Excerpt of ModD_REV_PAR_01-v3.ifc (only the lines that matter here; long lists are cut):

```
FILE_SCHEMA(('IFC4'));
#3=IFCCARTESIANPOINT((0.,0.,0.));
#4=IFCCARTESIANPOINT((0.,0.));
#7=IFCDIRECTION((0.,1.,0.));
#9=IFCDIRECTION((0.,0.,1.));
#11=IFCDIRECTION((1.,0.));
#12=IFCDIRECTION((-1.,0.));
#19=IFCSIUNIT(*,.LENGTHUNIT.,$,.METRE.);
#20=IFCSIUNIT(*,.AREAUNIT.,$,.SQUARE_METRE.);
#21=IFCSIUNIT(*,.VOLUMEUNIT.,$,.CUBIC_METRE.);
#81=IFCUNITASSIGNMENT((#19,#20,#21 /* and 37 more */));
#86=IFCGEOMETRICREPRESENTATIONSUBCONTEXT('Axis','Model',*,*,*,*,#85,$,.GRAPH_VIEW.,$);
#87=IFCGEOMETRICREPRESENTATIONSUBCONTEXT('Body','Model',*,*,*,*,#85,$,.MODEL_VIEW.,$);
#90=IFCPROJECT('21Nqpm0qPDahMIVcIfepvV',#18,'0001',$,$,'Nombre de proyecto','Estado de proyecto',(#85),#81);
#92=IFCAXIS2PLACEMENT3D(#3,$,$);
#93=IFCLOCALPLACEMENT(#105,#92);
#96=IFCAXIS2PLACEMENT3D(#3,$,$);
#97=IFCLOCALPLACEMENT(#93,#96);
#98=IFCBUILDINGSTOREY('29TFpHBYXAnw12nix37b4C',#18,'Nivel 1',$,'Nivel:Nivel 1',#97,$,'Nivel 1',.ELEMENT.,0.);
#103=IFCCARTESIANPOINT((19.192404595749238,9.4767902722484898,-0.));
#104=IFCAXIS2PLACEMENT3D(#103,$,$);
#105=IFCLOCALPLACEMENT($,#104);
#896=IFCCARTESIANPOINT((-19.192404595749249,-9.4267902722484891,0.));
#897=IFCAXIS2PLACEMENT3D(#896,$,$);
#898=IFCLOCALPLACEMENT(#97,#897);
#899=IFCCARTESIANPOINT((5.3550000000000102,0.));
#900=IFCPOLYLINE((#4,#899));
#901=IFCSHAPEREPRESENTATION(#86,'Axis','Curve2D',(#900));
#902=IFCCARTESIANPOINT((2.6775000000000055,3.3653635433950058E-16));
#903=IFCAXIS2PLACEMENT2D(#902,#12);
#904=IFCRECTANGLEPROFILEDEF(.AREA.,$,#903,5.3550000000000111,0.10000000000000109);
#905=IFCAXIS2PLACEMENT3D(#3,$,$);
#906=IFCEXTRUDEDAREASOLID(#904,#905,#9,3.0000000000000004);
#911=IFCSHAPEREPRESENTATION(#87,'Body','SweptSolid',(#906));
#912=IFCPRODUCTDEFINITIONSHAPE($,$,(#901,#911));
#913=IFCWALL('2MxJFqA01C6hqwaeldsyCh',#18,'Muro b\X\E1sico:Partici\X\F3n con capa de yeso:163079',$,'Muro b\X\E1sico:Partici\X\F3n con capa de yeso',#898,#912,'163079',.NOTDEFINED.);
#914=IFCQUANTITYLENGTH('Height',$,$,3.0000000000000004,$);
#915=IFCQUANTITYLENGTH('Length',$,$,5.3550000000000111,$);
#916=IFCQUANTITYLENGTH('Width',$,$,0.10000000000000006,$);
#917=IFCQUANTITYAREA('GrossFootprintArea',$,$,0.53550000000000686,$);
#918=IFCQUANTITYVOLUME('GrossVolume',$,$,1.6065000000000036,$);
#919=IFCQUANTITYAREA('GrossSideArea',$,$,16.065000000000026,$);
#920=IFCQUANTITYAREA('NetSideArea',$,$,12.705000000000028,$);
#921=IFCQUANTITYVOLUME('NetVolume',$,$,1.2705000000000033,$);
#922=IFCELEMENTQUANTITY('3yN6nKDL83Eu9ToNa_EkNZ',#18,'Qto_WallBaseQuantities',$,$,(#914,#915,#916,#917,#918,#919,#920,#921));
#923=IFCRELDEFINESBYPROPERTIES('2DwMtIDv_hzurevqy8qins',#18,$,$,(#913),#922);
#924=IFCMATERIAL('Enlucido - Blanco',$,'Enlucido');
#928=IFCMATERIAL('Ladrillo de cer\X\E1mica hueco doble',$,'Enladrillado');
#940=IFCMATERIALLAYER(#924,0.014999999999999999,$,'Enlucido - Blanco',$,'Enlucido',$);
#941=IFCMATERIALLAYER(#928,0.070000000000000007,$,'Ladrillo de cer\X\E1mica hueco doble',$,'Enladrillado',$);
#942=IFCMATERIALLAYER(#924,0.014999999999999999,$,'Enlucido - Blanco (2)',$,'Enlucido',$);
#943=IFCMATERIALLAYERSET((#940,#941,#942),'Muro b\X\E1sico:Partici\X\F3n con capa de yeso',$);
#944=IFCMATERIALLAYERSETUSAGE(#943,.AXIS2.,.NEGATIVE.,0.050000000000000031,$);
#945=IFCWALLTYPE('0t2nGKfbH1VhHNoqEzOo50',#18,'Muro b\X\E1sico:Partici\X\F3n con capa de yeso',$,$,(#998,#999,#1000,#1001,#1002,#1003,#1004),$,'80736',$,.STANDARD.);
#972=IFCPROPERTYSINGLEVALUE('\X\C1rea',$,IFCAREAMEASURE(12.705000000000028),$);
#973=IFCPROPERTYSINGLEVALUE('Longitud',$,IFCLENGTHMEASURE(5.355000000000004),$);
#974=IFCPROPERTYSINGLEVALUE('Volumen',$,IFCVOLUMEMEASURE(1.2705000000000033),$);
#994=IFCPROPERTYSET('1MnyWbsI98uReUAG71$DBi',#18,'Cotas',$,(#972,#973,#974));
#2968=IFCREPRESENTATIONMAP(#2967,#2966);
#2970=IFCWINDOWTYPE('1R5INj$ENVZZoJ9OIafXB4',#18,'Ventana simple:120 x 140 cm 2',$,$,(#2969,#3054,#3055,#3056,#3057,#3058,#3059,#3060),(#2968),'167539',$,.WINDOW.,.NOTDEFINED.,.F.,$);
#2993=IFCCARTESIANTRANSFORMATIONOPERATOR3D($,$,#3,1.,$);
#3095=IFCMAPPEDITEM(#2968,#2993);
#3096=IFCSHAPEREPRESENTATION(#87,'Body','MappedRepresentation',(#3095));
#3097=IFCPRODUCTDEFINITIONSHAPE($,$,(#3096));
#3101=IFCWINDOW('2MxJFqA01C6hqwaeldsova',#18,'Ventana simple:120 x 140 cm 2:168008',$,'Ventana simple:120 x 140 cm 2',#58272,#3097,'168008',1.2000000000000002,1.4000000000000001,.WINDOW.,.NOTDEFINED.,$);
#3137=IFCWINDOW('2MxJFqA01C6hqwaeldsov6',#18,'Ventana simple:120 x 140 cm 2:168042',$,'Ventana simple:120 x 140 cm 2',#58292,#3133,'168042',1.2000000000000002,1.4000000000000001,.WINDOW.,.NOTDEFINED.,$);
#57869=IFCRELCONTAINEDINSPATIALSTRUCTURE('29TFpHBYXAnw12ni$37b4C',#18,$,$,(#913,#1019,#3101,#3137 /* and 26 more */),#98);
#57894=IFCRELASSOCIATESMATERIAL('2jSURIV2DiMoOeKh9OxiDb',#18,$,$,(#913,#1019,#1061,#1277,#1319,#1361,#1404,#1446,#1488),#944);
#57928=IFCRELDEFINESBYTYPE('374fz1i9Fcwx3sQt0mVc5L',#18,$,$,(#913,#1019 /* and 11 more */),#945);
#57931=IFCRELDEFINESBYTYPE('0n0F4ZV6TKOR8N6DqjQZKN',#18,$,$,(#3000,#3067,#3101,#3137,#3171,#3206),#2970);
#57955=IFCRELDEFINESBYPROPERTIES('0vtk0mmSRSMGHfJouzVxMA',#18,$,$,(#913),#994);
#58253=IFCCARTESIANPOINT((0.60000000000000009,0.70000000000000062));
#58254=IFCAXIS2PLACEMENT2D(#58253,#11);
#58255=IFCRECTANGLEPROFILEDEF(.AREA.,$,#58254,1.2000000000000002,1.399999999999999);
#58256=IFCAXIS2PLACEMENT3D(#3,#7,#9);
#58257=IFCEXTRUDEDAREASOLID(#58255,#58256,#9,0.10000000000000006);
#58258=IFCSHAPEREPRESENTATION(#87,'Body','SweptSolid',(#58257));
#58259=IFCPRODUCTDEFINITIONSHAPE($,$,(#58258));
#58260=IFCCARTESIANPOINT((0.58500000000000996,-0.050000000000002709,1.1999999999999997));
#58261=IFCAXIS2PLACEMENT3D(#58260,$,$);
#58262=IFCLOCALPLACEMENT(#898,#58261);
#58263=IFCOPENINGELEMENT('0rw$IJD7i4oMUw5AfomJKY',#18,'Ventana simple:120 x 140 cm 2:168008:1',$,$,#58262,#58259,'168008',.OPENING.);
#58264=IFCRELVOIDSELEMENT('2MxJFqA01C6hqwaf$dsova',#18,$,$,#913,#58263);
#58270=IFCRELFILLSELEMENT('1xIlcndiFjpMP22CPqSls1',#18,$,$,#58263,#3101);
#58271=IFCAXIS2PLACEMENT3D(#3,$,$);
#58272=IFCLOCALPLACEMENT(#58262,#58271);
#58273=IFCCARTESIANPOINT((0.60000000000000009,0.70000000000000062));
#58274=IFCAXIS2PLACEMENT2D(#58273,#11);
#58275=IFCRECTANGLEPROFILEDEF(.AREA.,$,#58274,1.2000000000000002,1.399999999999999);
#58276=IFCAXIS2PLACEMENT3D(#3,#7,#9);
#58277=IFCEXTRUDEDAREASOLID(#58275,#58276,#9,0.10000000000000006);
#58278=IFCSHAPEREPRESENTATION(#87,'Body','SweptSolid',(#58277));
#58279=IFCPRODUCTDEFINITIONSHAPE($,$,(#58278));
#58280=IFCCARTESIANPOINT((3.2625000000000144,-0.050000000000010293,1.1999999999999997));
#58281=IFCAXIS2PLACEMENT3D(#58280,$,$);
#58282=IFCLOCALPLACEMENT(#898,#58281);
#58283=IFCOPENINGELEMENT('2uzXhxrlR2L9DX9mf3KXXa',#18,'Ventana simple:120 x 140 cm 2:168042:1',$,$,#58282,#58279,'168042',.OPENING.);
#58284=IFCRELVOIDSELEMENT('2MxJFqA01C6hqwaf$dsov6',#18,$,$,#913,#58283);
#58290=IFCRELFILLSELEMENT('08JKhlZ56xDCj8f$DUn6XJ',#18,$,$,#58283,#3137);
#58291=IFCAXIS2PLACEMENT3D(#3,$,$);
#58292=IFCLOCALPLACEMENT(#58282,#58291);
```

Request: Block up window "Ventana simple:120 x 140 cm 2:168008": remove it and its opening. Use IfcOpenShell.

```python
import ifcopenshell
import ifcopenshell.api.feature
import ifcopenshell.api.pset
import ifcopenshell.api.root
import ifcopenshell.geom
import ifcopenshell.util.element
import ifcopenshell.util.shape
import ifcopenshell.util.unit

model = ifcopenshell.open("ModD_REV_PAR_01-v3.ifc")
area_scale = ifcopenshell.util.unit.calculate_unit_scale(model, "AREAUNIT")
volume_scale = ifcopenshell.util.unit.calculate_unit_scale(model, "VOLUMEUNIT")
settings = ifcopenshell.geom.settings()


def volume(element):
    """Net volume in cubic metres, openings subtracted."""
    shape = ifcopenshell.geom.create_shape(settings, element)
    return ifcopenshell.util.shape.get_volume(shape.geometry)


window = model.by_id(3101)
opening = window.FillsVoids[0].RelatingOpeningElement
wall = opening.VoidsElements[0].RelatingBuildingElement
before = volume(wall)

ifcopenshell.api.root.remove_product(model, product=window)
ifcopenshell.api.feature.remove_feature(model, feature=opening)

after = volume(wall)
thickness = 0.1  # wall thickness in metres

# Update the wall's stored quantities.
qto = model.by_id(ifcopenshell.util.element.get_pset(wall, "Qto_WallBaseQuantities", should_inherit=False)["id"])
ifcopenshell.api.pset.edit_qto(model, qto=qto, properties={
    "NetSideArea": after / thickness / area_scale,
    "NetVolume": after / volume_scale,
})
pset = model.by_id(ifcopenshell.util.element.get_pset(wall, "Cotas", should_inherit=False)["id"])
ifcopenshell.api.pset.edit_pset(model, pset=pset, properties={
    "Área": model.create_entity("IfcAreaMeasure", after / thickness / area_scale),
    "Volumen": model.create_entity("IfcVolumeMeasure", after / volume_scale),
})

print(f"wall volume {before:.3f} -> {after:.3f} m3")

model.write("ModD_REV_PAR_01-v3_v2.ifc")
```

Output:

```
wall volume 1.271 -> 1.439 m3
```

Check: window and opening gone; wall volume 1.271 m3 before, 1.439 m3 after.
